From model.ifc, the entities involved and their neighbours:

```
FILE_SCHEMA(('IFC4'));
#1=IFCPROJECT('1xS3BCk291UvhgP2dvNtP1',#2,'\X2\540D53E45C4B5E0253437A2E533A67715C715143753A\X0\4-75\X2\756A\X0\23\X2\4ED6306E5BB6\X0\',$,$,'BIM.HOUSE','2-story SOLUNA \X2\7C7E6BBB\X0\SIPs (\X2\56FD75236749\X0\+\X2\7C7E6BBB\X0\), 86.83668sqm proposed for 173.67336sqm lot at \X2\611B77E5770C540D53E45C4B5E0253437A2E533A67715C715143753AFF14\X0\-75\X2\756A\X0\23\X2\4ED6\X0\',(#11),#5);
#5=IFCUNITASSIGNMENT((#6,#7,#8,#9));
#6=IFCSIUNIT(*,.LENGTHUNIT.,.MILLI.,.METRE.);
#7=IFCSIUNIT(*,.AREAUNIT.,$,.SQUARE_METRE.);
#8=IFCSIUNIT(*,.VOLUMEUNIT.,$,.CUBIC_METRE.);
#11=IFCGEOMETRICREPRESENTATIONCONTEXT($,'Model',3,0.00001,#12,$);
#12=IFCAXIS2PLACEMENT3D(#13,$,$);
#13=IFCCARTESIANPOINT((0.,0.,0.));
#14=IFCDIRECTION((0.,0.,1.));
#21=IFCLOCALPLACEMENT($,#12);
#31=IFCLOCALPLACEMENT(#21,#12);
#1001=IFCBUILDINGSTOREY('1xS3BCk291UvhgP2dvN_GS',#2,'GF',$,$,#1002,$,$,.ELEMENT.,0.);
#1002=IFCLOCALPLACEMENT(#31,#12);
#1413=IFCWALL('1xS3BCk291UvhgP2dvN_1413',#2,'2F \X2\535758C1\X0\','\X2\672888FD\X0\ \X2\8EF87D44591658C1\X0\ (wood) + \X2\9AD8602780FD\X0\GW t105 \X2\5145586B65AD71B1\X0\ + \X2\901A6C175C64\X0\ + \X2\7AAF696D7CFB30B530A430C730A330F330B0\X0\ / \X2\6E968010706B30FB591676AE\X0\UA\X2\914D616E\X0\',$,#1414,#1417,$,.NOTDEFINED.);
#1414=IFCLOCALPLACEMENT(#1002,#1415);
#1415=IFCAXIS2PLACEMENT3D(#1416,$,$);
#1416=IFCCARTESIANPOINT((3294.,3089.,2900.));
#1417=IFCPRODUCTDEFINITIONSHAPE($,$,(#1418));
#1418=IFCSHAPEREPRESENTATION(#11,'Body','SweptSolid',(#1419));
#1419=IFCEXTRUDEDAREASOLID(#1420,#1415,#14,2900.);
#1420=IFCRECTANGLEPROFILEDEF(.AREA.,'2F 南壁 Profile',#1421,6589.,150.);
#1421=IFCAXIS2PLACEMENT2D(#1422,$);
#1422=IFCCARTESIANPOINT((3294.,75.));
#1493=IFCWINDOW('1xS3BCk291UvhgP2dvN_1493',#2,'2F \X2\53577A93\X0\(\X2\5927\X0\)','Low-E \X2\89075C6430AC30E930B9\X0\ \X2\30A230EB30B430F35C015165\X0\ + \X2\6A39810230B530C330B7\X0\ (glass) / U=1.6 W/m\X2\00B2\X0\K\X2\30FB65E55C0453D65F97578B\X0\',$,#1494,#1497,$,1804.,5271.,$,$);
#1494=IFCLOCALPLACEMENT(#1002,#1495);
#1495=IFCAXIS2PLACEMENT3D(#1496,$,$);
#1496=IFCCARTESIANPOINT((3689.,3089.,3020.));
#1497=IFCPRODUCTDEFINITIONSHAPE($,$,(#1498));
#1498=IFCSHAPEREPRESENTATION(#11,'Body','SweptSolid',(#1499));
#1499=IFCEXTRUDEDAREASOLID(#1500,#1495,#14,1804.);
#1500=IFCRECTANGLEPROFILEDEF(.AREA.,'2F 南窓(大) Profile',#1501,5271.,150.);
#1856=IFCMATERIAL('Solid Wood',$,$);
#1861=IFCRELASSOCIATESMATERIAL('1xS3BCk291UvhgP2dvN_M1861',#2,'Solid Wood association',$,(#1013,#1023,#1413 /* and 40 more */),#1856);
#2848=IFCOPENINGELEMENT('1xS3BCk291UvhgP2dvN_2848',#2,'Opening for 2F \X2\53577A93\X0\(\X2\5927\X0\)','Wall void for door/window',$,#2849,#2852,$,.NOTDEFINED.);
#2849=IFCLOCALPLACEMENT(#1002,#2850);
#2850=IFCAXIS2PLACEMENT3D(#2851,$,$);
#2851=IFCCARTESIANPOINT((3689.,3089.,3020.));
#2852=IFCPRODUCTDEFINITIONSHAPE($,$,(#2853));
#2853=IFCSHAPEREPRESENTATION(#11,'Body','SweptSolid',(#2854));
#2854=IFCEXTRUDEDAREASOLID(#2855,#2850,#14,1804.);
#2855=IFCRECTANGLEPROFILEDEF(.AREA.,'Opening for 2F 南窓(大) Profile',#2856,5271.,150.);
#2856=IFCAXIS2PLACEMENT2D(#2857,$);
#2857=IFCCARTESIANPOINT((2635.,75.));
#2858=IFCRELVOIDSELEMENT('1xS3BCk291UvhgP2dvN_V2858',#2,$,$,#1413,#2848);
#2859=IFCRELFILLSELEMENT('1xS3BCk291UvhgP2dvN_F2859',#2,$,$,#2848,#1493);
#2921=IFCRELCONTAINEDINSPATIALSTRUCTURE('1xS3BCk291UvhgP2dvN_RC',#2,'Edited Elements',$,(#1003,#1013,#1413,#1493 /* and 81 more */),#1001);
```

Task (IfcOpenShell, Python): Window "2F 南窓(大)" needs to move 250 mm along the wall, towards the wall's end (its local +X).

```python
import ifcopenshell
import ifcopenshell.api.geometry
import ifcopenshell.util.placement

model = ifcopenshell.open("model.ifc")

window = model.by_id(1493)
opening = window.FillsVoids[0].RelatingOpeningElement
wall = opening.VoidsElements[0].RelatingBuildingElement

wall_matrix = ifcopenshell.util.placement.get_local_placement(wall.ObjectPlacement)
shift = wall_matrix[:3, 0] * 250.0
before = ifcopenshell.util.placement.get_local_placement(window.ObjectPlacement)[:3, 3].copy()

# The window is not placed relative to its opening, so move both.
for product in (opening, window):
    matrix = ifcopenshell.util.placement.get_local_placement(product.ObjectPlacement)
    matrix[:3, 3] += shift
    ifcopenshell.api.geometry.edit_object_placement(model, product=product, matrix=matrix, is_si=False)

after = ifcopenshell.util.placement.get_local_placement(window.ObjectPlacement)[:3, 3]
print("window moved by", (after - before).round(3) + 0.0)

model.write("model_v2.ifc")
```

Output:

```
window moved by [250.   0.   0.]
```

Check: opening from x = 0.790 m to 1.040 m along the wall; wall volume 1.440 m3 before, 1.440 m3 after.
